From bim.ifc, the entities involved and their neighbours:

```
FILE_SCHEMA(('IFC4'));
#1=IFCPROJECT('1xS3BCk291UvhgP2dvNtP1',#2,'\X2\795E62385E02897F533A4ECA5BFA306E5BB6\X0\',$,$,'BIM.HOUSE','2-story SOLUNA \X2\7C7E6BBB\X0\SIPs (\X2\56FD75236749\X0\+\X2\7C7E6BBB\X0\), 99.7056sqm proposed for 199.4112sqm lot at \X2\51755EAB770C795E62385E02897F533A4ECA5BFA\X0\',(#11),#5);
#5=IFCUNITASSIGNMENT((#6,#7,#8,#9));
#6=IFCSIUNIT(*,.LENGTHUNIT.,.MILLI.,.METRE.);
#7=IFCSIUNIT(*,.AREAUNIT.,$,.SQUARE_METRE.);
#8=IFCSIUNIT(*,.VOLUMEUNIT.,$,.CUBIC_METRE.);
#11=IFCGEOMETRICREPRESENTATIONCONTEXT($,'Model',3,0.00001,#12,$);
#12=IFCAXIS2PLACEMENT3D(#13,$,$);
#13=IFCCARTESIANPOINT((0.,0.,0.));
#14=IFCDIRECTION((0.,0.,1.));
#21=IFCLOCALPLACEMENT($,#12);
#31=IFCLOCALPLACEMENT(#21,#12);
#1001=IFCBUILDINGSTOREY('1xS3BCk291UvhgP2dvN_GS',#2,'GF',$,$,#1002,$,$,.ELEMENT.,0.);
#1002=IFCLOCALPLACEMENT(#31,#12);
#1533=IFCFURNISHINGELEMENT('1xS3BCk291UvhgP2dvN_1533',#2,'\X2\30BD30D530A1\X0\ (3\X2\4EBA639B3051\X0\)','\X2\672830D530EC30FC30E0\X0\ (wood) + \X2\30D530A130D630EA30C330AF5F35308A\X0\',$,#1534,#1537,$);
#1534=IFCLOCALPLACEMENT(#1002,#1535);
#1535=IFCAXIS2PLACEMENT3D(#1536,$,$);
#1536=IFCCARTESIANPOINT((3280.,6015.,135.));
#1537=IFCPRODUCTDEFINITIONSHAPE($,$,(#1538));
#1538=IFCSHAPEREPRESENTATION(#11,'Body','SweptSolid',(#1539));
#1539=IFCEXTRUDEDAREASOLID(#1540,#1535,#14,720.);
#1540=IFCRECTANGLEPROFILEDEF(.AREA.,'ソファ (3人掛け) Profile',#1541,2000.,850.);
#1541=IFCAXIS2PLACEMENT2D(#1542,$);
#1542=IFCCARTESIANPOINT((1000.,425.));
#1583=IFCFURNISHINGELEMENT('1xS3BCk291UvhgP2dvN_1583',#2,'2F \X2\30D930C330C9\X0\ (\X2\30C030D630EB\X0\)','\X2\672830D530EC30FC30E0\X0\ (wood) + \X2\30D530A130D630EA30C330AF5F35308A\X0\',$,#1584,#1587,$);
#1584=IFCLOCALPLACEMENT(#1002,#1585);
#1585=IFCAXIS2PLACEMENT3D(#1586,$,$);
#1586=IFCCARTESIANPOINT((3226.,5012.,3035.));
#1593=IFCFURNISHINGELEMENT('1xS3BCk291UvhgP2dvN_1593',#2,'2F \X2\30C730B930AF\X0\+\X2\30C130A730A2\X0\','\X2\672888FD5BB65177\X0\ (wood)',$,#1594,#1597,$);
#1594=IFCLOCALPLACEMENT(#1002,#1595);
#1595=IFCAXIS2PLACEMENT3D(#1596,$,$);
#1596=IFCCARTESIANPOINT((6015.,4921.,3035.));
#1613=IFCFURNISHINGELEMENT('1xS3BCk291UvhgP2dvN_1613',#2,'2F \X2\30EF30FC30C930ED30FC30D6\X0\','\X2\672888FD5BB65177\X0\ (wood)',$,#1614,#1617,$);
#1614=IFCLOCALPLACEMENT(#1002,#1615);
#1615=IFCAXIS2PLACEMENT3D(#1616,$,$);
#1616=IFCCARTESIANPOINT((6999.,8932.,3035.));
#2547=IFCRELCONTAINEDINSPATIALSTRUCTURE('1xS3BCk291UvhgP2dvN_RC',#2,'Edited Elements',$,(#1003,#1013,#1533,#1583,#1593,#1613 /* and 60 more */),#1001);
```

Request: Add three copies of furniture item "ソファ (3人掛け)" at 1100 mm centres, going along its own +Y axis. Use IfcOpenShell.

```python
import ifcopenshell
import ifcopenshell.api.geometry
import ifcopenshell.api.root
import ifcopenshell.util.element
import ifcopenshell.util.placement
import ifcopenshell.util.unit

model = ifcopenshell.open("bim.ifc")
unit_scale = ifcopenshell.util.unit.calculate_unit_scale(model)


def reuse_history(source, copy):
    """copy_class also copies each property set's owner history, people and application; keep the originals."""
    for rel in copy.IsDefinedBy:
        if rel.is_a("IfcRelDefinesByProperties") and (history := rel.RelatingPropertyDefinition.OwnerHistory):
            rel.RelatingPropertyDefinition.OwnerHistory = source.OwnerHistory
            ifcopenshell.util.element.remove_deep2(model, history)


source = model.by_guid("1xS3BCk291UvhgP2dvN_1533")
base = ifcopenshell.util.placement.get_local_placement(source.ObjectPlacement)
step = base[:3, 1] * 1.1 / unit_scale

for i in range(1, 4):
    copy = ifcopenshell.api.root.copy_class(model, product=source)
    copy.Representation = ifcopenshell.util.element.copy_deep(
        model, source.Representation, exclude=["IfcGeometricRepresentationContext", "IfcRepresentationMap"]
    )
    reuse_history(source, copy)
    matrix = base.copy()
    matrix[:3, 3] += i * step
    print("added at", matrix[:3, 3].round(3) + 0.0)
    ifcopenshell.api.geometry.edit_object_placement(model, product=copy, matrix=matrix, is_si=False)

model.write("bim_rev.ifc")
```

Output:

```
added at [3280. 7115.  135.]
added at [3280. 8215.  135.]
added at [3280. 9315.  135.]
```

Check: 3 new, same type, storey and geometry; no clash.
